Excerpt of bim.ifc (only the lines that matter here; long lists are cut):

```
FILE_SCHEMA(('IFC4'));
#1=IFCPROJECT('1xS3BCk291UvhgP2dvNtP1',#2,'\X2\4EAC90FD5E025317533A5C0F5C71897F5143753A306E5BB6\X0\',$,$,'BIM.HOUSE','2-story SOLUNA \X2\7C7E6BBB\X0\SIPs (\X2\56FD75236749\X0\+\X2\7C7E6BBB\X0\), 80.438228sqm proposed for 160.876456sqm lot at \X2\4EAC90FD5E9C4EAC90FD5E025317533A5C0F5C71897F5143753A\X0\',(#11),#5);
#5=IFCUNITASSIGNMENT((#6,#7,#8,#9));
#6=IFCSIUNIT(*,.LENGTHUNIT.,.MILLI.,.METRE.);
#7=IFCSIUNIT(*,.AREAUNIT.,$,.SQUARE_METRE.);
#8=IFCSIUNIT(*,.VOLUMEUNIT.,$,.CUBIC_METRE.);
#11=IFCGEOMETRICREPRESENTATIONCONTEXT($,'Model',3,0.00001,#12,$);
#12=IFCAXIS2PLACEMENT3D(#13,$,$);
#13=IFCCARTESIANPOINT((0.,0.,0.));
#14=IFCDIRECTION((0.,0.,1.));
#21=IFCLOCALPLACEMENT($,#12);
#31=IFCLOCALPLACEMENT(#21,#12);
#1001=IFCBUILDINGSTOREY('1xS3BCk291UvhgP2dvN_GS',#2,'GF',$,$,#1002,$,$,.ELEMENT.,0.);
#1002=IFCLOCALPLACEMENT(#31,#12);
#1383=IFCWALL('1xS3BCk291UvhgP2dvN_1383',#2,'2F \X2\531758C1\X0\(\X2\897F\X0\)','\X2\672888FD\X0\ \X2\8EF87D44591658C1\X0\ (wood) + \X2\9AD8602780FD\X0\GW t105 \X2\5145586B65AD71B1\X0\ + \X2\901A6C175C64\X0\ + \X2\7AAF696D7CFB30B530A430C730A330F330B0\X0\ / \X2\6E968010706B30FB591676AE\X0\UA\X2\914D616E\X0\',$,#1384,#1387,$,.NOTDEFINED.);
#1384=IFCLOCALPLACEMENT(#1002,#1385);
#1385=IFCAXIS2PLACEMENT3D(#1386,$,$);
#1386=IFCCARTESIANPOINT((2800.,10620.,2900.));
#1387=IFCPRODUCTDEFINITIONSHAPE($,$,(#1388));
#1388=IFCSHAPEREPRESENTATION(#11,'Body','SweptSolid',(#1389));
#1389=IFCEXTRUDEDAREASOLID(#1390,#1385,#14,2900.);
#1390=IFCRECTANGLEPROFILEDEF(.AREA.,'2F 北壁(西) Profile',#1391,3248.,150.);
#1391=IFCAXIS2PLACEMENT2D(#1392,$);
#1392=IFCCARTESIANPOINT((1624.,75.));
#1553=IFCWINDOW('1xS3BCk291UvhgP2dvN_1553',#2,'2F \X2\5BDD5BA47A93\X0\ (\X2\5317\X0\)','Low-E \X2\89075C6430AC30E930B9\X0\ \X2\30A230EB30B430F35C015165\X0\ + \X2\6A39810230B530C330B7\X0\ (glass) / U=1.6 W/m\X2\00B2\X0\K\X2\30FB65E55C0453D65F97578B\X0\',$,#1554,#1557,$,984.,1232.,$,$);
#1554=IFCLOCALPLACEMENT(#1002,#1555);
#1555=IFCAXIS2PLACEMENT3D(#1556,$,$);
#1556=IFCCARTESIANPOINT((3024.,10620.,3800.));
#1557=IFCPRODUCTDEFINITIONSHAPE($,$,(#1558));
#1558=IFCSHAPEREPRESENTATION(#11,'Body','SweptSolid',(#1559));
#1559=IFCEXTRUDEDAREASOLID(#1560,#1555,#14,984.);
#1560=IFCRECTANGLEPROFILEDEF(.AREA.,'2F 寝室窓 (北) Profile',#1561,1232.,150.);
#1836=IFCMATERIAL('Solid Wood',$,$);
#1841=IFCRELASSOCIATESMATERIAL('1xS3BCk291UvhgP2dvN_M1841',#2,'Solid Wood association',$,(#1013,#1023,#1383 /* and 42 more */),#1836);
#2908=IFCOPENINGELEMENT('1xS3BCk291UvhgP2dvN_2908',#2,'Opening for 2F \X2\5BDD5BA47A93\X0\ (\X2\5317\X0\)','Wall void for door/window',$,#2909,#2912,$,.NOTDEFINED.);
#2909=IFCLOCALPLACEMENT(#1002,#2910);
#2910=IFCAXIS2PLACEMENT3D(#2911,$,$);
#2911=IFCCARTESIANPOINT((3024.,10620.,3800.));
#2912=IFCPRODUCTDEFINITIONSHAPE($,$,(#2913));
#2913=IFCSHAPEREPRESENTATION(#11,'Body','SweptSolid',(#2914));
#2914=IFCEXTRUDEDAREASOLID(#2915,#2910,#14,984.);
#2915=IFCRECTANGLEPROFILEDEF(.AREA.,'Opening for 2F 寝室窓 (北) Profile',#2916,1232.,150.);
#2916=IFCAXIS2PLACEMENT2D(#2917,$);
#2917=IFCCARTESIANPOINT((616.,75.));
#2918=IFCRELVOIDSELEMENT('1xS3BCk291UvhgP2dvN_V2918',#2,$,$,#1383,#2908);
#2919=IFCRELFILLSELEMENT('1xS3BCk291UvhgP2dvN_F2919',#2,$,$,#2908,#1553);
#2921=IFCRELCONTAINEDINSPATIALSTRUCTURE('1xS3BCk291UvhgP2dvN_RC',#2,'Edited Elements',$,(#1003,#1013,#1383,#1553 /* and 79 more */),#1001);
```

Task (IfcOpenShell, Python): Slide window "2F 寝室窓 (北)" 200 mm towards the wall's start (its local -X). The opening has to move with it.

```python
import ifcopenshell
import ifcopenshell.api.geometry
import ifcopenshell.util.placement
import ifcopenshell.util.unit

model = ifcopenshell.open("bim.ifc")
unit_scale = ifcopenshell.util.unit.calculate_unit_scale(model)

window = model.by_guid("1xS3BCk291UvhgP2dvN_1553")
opening = window.FillsVoids[0].RelatingOpeningElement
wall = opening.VoidsElements[0].RelatingBuildingElement

wall_matrix = ifcopenshell.util.placement.get_local_placement(wall.ObjectPlacement)
shift = wall_matrix[:3, 0] * -0.2 / unit_scale
before = ifcopenshell.util.placement.get_local_placement(window.ObjectPlacement)[:3, 3].copy()

# The window is not placed relative to its opening, so move both.
for product in (opening, window):
    matrix = ifcopenshell.util.placement.get_local_placement(product.ObjectPlacement)
    matrix[:3, 3] += shift
    ifcopenshell.api.geometry.edit_object_placement(model, product=product, matrix=matrix, is_si=False)

after = ifcopenshell.util.placement.get_local_placement(window.ObjectPlacement)[:3, 3]
print("window moved by", (after - before).round(3) + 0.0)

model.write("bim_edited.ifc")
```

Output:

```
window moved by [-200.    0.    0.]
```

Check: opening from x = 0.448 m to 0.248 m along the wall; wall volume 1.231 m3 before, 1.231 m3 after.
